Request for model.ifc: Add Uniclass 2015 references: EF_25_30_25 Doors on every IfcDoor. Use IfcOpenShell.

First a look at what the model holds.

```python
import ifcopenshell

model = ifcopenshell.open("model.ifc")
print(model.schema)
print("classifications:", [c.Name for c in model.by_type("IfcClassification")])
for ifc_class in ("IfcDoor", "IfcRoof", "IfcStair", "IfcWall", "IfcWindow"):
    print(ifc_class, len(model.by_type(ifc_class)))
```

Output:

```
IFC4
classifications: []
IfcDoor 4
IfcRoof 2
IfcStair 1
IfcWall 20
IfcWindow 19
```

```python
import ifcopenshell
import ifcopenshell.api.classification

model = ifcopenshell.open("model.ifc")

system = ifcopenshell.api.classification.add_classification(model, classification="Uniclass 2015")

codes = {
    "IfcDoor": ("EF_25_30_25", "Doors"),
}
for ifc_class, (code, name) in codes.items():
    products = model.by_type(ifc_class)
    ifcopenshell.api.classification.add_reference(
        model, products=products, classification=system, identification=code, name=name
    )
    print(code, len(products))

model.write("model_rev.ifc")
```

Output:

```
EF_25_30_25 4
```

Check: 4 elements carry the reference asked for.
